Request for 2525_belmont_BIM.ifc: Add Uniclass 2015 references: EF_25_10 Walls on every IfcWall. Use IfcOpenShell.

First a look at what the model holds.

```python
import ifcopenshell

model = ifcopenshell.open("2525_belmont_BIM.ifc")
print(model.schema)
print("classifications:", [c.Name for c in model.by_type("IfcClassification")])
for ifc_class in ("IfcDoor", "IfcRoof", "IfcStair", "IfcWall", "IfcWindow"):
    print(ifc_class, len(model.by_type(ifc_class)))
```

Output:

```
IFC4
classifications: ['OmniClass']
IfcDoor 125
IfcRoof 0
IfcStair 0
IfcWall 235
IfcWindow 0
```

```python
import ifcopenshell
import ifcopenshell.api.classification

model = ifcopenshell.open("2525_belmont_BIM.ifc")

system = ifcopenshell.api.classification.add_classification(model, classification="Uniclass 2015")

codes = {
    "IfcWall": ("EF_25_10", "Walls"),
}
for ifc_class, (code, name) in codes.items():
    products = model.by_type(ifc_class)
    ifcopenshell.api.classification.add_reference(
        model, products=products, classification=system, identification=code, name=name
    )
    print(code, len(products))

model.write("2525_belmont_BIM_rev.ifc")
```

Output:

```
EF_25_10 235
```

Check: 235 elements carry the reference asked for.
